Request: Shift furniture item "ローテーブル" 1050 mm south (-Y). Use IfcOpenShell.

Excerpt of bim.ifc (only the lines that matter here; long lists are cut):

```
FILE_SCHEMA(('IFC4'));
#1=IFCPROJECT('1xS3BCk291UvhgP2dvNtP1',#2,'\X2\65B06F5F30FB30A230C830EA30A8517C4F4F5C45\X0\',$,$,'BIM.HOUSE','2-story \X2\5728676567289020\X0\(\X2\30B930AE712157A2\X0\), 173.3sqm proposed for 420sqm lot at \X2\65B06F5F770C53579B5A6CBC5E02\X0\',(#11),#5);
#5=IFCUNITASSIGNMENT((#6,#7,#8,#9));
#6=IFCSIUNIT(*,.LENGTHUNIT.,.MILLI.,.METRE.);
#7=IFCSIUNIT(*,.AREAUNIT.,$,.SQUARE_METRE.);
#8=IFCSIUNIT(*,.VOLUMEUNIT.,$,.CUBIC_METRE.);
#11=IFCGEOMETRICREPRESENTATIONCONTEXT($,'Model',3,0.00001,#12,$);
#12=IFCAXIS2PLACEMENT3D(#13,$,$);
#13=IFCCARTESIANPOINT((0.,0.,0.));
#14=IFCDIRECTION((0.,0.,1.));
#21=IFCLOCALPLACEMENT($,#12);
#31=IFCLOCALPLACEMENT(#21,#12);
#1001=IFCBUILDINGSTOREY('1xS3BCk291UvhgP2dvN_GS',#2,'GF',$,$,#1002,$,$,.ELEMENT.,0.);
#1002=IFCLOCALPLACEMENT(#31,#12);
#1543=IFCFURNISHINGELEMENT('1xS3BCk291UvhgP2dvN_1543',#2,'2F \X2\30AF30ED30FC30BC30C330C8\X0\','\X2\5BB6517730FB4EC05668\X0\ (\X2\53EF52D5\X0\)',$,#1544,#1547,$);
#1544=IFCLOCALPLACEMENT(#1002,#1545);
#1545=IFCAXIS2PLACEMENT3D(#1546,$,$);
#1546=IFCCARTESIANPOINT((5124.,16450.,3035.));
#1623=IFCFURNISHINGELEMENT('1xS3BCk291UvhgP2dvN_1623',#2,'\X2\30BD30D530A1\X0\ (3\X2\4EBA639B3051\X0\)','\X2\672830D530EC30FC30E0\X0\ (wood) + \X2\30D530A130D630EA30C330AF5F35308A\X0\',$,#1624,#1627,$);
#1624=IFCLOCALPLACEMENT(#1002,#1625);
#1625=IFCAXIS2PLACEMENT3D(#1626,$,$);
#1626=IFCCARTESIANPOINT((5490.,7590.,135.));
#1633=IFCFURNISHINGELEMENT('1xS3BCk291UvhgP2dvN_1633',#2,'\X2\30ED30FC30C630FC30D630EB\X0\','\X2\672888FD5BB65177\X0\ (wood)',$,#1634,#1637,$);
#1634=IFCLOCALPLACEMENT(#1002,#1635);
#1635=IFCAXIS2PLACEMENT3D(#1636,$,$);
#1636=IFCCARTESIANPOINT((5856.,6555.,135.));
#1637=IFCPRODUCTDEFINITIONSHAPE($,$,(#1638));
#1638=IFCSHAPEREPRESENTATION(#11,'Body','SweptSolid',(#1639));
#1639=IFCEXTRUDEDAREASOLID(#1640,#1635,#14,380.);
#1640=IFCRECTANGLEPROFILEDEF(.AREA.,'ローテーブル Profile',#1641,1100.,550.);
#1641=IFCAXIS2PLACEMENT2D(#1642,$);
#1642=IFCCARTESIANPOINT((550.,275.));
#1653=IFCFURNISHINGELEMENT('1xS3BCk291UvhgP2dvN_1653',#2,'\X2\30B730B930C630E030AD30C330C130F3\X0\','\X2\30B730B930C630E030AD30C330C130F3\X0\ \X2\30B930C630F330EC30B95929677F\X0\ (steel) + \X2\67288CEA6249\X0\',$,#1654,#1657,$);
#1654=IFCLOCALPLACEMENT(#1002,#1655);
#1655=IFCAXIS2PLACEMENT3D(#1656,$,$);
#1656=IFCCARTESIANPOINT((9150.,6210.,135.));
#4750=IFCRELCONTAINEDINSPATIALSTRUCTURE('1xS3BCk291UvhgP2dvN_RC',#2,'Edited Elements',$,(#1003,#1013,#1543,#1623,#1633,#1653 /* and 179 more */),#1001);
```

```python
import ifcopenshell
import ifcopenshell.api.geometry
import ifcopenshell.util.placement

model = ifcopenshell.open("bim.ifc")

item = model.by_id(1633)
matrix = ifcopenshell.util.placement.get_local_placement(item.ObjectPlacement)
matrix[1, 3] -= 1050.0
ifcopenshell.api.geometry.edit_object_placement(model, product=item, matrix=matrix, is_si=False)

print(ifcopenshell.util.placement.get_local_placement(item.ObjectPlacement).round(3) + 0.0)

model.write("bim_updated.ifc")
```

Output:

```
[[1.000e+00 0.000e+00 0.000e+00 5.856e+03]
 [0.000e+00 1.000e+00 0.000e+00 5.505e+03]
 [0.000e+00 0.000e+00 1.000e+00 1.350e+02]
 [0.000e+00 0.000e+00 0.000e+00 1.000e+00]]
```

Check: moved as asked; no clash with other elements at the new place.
